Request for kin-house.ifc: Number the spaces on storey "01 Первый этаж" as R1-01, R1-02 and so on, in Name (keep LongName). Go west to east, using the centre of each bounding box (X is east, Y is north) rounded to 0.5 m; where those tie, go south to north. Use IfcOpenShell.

First a look at what the model holds.

```python
import ifcopenshell
import ifcopenshell.util.element
import ifcopenshell.util.placement

model = ifcopenshell.open("kin-house.ifc")
print(model.schema)
storey = next(s for s in model.by_type("IfcBuildingStorey") if s.Name == "01 Первый этаж")
spaces = [e for e in ifcopenshell.util.element.get_decomposition(storey) if e.is_a("IfcSpace")]
for e in sorted(spaces, key=lambda e: e.id()):
    origin = ifcopenshell.util.placement.get_local_placement(e.ObjectPlacement)[:3, 3]
    print(e.id(), e.Name, e.LongName, origin.round(2) + 0.0, sep=" | ")
```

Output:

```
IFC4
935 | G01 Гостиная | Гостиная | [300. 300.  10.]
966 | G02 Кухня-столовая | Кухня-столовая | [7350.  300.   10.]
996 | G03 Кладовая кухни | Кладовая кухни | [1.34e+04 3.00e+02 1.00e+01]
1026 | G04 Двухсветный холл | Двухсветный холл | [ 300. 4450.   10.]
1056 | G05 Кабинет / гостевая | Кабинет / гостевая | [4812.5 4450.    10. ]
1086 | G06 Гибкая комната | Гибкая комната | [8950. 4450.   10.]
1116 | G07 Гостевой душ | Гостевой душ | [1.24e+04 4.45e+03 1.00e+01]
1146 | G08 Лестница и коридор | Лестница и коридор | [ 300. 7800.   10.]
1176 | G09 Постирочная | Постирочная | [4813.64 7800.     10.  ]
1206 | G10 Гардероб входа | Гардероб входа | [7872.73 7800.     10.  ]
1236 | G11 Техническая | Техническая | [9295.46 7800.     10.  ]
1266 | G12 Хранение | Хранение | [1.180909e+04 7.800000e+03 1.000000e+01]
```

```python
import ifcopenshell
import ifcopenshell.geom
import ifcopenshell.util.element
import ifcopenshell.util.shape

model = ifcopenshell.open("kin-house.ifc")
settings = ifcopenshell.geom.settings()
settings.set("use-world-coords", True)


def centre(element):
    shape = ifcopenshell.geom.create_shape(settings, element)
    return ifcopenshell.util.shape.get_bbox_centroid(shape.geometry)


storey = next(s for s in model.by_type("IfcBuildingStorey") if s.Name == "01 Первый этаж")
spaces = [e for e in ifcopenshell.util.element.get_decomposition(storey) if e.is_a("IfcSpace")]

# Insertion points can sit at a corner or the storey origin, so sort by the geometry (in metres).
centres = {e: centre(e) for e in spaces}
spaces.sort(key=lambda e: (round(centres[e][0] / 0.5), centres[e][1]))

for i, e in enumerate(spaces, start=1):
    number = f"R1-{i:02d}"
    e.Name = number
    print(e.id(), number)

model.write("kin-house_v2.ifc")
```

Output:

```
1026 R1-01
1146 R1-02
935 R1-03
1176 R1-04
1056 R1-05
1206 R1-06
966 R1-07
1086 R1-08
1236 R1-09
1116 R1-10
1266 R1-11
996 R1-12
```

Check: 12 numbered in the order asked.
